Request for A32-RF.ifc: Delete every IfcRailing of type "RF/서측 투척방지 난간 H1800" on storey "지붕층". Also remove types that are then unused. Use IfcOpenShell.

First a look at what the model holds.

```python
import ifcopenshell
import ifcopenshell.util.element

model = ifcopenshell.open("A32-RF.ifc")
print(model.schema)
storey = next(s for s in model.by_type("IfcBuildingStorey") if s.Name == "지붕층")
railings = [e for e in ifcopenshell.util.element.get_decomposition(storey) if e.is_a("IfcRailing")]
seen = {}
for e in railings:
    element_type = ifcopenshell.util.element.get_type(e)
    name = element_type.Name if element_type not in (None, e) else None
    seen[name] = seen.get(name, 0) + 1
for name, count in sorted(seen.items(), key=str):
    print(count, "x", name)
```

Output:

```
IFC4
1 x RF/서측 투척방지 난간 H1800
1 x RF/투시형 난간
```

```python
import ifcopenshell
import ifcopenshell.api.root
import ifcopenshell.util.element

model = ifcopenshell.open("A32-RF.ifc")

storey = next(s for s in model.by_type("IfcBuildingStorey") if s.Name == "지붕층")
railings = [e for e in ifcopenshell.util.element.get_decomposition(storey) if e.is_a("IfcRailing")]
targets = [e for e in railings if (t := ifcopenshell.util.element.get_type(e)) not in (None, e) and t.Name == "RF/서측 투척방지 난간 H1800"]
types = {ifcopenshell.util.element.get_type(e) for e in targets} - {None, *targets}

for e in targets:
    ifcopenshell.api.root.remove_product(model, product=e)
print(len(targets), "removed")

unused = [t for t in types if not ifcopenshell.util.element.get_types(t)]
for t in unused:
    ifcopenshell.api.root.remove_product(model, product=t)
print(len(unused), "unused types removed")

model.write("A32-RF_rev.ifc")
```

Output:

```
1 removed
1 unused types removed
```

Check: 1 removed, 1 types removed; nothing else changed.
